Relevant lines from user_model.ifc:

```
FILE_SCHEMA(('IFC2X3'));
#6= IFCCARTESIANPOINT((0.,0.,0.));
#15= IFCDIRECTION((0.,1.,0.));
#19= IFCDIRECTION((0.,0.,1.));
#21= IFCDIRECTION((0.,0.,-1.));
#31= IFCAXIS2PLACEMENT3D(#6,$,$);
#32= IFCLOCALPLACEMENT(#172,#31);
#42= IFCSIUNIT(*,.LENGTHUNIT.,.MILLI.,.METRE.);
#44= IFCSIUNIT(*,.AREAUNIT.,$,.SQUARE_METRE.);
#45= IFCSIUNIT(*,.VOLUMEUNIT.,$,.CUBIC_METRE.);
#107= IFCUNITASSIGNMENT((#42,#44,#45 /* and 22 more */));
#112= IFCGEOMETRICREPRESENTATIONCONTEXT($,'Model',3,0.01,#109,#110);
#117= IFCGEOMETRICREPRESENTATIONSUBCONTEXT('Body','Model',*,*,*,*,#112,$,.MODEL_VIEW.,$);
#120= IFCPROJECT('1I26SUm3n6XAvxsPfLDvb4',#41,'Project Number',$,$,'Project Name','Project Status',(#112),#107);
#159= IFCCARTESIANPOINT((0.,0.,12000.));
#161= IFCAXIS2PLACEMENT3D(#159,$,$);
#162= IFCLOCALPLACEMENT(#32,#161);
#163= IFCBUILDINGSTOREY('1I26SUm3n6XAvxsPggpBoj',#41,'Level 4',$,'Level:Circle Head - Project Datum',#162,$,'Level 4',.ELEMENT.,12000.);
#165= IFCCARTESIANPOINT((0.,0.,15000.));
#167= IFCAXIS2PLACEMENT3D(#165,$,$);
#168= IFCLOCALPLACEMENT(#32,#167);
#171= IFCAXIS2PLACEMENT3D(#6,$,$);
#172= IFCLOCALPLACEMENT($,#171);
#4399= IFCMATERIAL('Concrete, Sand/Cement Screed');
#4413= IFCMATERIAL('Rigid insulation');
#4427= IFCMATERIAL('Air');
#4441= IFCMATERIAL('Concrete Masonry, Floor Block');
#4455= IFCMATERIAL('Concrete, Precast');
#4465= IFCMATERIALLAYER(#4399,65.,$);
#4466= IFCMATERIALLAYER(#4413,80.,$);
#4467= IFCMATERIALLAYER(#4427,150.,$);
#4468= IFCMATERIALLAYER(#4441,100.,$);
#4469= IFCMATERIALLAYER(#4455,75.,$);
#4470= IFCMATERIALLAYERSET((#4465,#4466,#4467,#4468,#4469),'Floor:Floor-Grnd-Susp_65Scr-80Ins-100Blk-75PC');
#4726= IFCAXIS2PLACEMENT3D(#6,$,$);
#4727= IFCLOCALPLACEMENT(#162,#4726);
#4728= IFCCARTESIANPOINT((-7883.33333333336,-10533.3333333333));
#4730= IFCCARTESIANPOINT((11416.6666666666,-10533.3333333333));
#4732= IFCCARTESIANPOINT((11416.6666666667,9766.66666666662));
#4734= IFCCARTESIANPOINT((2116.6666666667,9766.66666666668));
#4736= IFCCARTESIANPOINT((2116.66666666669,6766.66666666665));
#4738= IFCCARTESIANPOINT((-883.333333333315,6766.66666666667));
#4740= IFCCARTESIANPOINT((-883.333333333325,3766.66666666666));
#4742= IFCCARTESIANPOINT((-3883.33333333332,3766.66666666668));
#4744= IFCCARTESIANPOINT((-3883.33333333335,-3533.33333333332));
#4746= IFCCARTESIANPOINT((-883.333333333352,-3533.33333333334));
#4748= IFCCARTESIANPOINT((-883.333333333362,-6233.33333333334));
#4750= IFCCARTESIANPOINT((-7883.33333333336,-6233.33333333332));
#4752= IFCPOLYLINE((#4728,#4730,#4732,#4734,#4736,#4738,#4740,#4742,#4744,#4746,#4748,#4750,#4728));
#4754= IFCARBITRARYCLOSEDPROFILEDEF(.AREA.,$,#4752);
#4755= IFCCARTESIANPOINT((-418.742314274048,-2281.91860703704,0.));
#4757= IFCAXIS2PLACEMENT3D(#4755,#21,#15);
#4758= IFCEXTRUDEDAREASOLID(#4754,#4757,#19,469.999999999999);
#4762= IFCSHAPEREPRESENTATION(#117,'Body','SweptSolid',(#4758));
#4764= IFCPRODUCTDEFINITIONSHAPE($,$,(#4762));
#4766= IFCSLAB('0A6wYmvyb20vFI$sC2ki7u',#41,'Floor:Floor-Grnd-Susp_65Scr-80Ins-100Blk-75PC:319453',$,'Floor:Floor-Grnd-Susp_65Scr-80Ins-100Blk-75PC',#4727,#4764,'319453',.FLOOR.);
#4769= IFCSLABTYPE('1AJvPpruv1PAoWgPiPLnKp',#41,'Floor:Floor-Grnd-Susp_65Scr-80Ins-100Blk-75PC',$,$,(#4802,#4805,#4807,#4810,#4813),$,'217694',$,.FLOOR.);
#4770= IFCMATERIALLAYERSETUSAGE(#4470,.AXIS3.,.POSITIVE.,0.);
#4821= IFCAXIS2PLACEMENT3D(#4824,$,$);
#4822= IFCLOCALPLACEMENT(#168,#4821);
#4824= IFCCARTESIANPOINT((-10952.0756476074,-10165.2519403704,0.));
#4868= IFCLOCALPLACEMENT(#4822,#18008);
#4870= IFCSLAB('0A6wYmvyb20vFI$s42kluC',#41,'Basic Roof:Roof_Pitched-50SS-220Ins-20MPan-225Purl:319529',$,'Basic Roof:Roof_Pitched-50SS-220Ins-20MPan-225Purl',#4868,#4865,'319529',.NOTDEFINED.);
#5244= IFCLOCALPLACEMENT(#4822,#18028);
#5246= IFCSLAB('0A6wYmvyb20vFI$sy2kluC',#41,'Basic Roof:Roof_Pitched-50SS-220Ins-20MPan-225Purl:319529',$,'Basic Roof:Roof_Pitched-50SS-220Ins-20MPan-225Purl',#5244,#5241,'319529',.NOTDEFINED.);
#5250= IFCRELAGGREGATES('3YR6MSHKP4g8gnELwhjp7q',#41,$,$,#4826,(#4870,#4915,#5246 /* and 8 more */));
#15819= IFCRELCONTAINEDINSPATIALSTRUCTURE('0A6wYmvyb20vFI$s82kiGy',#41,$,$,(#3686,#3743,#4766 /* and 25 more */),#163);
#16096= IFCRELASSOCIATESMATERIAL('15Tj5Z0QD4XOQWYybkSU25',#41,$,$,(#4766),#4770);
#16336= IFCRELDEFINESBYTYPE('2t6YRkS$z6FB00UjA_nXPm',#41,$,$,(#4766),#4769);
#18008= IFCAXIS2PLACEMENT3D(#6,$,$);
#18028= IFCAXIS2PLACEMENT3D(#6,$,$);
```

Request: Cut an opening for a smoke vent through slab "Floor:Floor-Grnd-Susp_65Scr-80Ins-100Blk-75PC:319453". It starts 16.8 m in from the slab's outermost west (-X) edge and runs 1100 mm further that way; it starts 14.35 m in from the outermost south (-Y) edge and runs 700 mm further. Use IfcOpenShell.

```python
import numpy as np
import ifcopenshell
import ifcopenshell.api.feature
import ifcopenshell.api.geometry
import ifcopenshell.api.root
import ifcopenshell.geom
import ifcopenshell.util.placement
import ifcopenshell.util.representation
import ifcopenshell.util.shape
import ifcopenshell.util.unit

model = ifcopenshell.open("user_model.ifc")
unit_scale = ifcopenshell.util.unit.calculate_unit_scale(model)
settings = ifcopenshell.geom.settings()


def volume(element):
    """Net volume in cubic metres, openings subtracted."""
    shape = ifcopenshell.geom.create_shape(settings, element)
    return ifcopenshell.util.shape.get_volume(shape.geometry)


slab = model.by_id(4766)
before = volume(slab)

# Extent in the slab's own axes, in metres. The edges named are its -X and -Y sides.
slab_shape = ifcopenshell.geom.create_shape(settings, slab)
vertices = ifcopenshell.util.shape.get_vertices(slab_shape.geometry)
x_min, y_min, bottom = vertices.min(axis=0)
top = vertices[:, 2].max()

opening = ifcopenshell.api.root.create_entity(model, ifc_class="IfcOpeningElement", name="Smoke vent opening")
context = ifcopenshell.util.representation.get_context(model, "Model", "Body", "MODEL_VIEW")
width, depth = 1.1, 0.7
outline = [(0.0, 0.0), (width, 0.0), (width, depth), (0.0, depth), (0.0, 0.0)]
# Overshoot both faces by 50 mm so the cut is clean.
shape = ifcopenshell.api.geometry.add_slab_representation(
    model, context=context, depth=top - bottom + 0.1, polyline=outline
)
ifcopenshell.api.geometry.assign_representation(model, product=opening, representation=shape)

matrix = ifcopenshell.util.placement.get_local_placement(slab.ObjectPlacement)
matrix[:, 3] = matrix @ np.append(np.array([x_min + 16.8, y_min + 14.35, bottom - 0.05]) / unit_scale, 1.0)
ifcopenshell.api.geometry.edit_object_placement(model, product=opening, matrix=matrix, is_si=False)
ifcopenshell.api.feature.add_feature(model, feature=opening, element=slab)

after = volume(slab)

print(f"slab volume {before:.3f} -> {after:.3f} m3")

model.write("user_model_updated.ifc")
```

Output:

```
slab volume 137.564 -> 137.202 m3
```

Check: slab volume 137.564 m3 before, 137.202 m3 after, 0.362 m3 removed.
